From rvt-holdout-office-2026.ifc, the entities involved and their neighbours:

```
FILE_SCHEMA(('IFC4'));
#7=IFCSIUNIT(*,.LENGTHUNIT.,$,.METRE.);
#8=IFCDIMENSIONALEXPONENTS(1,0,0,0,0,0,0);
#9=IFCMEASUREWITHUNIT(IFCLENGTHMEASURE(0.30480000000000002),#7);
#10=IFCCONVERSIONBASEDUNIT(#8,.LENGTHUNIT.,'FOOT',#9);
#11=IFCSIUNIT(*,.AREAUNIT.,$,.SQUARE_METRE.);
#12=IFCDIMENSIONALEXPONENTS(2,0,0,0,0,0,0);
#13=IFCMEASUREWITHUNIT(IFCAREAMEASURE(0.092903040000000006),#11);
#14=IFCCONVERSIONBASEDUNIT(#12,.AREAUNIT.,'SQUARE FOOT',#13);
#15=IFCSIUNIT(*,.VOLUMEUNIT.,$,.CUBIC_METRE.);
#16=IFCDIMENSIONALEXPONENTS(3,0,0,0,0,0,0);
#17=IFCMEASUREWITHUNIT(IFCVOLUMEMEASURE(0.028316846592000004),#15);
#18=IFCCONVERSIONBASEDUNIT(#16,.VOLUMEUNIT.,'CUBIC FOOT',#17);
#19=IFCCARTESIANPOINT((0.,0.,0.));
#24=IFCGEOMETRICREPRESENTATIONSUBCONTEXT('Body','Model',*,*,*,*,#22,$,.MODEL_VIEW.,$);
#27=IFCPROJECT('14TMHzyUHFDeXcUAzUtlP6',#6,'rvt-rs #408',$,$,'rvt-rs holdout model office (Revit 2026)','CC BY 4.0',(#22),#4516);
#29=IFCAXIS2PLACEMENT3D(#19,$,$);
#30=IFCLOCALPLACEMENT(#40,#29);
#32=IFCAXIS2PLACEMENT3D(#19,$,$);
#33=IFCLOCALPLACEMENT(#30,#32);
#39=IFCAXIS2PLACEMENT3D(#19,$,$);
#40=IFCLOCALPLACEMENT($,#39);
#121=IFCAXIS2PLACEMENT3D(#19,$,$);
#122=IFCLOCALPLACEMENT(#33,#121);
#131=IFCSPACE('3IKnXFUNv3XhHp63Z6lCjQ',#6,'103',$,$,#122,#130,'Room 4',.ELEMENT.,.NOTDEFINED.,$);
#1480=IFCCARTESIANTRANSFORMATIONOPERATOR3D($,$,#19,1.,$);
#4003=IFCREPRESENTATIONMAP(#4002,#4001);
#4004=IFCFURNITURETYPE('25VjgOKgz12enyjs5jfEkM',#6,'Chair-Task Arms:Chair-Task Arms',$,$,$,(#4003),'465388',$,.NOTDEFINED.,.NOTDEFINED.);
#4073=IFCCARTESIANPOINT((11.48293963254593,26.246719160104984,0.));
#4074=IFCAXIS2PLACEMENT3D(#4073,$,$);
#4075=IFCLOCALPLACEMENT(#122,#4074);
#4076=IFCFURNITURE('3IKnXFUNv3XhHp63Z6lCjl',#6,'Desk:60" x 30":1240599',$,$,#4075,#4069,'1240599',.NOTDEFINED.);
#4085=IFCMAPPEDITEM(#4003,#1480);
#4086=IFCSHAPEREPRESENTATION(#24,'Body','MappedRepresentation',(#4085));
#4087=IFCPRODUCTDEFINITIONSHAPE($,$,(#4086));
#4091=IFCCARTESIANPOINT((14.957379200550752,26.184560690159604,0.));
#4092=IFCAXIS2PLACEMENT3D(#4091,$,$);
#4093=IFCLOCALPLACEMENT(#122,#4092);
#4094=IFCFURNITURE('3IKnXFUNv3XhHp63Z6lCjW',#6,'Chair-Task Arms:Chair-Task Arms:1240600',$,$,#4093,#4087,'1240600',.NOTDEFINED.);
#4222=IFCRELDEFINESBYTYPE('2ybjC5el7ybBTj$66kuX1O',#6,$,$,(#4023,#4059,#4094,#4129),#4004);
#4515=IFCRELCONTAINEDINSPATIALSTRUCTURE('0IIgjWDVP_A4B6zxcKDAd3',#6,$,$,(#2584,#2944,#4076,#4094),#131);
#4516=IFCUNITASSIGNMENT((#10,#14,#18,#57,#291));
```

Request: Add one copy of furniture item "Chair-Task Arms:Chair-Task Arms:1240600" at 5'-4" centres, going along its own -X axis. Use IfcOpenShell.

```python
import ifcopenshell
import ifcopenshell.api.geometry
import ifcopenshell.api.root
import ifcopenshell.util.element
import ifcopenshell.util.placement
import ifcopenshell.util.unit

model = ifcopenshell.open("rvt-holdout-office-2026.ifc")
unit_scale = ifcopenshell.util.unit.calculate_unit_scale(model)


def reuse_history(source, copy):
    """copy_class also copies each property set's owner history, people and application; keep the originals."""
    for rel in copy.IsDefinedBy:
        if rel.is_a("IfcRelDefinesByProperties") and (history := rel.RelatingPropertyDefinition.OwnerHistory):
            rel.RelatingPropertyDefinition.OwnerHistory = source.OwnerHistory
            ifcopenshell.util.element.remove_deep2(model, history)


source = model.by_guid("3IKnXFUNv3XhHp63Z6lCjW")
base = ifcopenshell.util.placement.get_local_placement(source.ObjectPlacement)
step = -base[:3, 0] * 64 * 0.0254 / unit_scale

for i in range(1, 2):
    copy = ifcopenshell.api.root.copy_class(model, product=source)
    copy.Representation = ifcopenshell.util.element.copy_deep(
        model, source.Representation, exclude=["IfcGeometricRepresentationContext", "IfcRepresentationMap"]
    )
    copy.Name = "Chair-Task Arms:Chair-Task Arms"
    copy.Tag = None
    reuse_history(source, copy)
    matrix = base.copy()
    matrix[:3, 3] += i * step
    print("added at", matrix[:3, 3].round(3) + 0.0)
    ifcopenshell.api.geometry.edit_object_placement(model, product=copy, matrix=matrix, is_si=False)

model.write("rvt-holdout-office-2026_edited.ifc")
```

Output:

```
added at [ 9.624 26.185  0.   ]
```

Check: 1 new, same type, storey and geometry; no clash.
